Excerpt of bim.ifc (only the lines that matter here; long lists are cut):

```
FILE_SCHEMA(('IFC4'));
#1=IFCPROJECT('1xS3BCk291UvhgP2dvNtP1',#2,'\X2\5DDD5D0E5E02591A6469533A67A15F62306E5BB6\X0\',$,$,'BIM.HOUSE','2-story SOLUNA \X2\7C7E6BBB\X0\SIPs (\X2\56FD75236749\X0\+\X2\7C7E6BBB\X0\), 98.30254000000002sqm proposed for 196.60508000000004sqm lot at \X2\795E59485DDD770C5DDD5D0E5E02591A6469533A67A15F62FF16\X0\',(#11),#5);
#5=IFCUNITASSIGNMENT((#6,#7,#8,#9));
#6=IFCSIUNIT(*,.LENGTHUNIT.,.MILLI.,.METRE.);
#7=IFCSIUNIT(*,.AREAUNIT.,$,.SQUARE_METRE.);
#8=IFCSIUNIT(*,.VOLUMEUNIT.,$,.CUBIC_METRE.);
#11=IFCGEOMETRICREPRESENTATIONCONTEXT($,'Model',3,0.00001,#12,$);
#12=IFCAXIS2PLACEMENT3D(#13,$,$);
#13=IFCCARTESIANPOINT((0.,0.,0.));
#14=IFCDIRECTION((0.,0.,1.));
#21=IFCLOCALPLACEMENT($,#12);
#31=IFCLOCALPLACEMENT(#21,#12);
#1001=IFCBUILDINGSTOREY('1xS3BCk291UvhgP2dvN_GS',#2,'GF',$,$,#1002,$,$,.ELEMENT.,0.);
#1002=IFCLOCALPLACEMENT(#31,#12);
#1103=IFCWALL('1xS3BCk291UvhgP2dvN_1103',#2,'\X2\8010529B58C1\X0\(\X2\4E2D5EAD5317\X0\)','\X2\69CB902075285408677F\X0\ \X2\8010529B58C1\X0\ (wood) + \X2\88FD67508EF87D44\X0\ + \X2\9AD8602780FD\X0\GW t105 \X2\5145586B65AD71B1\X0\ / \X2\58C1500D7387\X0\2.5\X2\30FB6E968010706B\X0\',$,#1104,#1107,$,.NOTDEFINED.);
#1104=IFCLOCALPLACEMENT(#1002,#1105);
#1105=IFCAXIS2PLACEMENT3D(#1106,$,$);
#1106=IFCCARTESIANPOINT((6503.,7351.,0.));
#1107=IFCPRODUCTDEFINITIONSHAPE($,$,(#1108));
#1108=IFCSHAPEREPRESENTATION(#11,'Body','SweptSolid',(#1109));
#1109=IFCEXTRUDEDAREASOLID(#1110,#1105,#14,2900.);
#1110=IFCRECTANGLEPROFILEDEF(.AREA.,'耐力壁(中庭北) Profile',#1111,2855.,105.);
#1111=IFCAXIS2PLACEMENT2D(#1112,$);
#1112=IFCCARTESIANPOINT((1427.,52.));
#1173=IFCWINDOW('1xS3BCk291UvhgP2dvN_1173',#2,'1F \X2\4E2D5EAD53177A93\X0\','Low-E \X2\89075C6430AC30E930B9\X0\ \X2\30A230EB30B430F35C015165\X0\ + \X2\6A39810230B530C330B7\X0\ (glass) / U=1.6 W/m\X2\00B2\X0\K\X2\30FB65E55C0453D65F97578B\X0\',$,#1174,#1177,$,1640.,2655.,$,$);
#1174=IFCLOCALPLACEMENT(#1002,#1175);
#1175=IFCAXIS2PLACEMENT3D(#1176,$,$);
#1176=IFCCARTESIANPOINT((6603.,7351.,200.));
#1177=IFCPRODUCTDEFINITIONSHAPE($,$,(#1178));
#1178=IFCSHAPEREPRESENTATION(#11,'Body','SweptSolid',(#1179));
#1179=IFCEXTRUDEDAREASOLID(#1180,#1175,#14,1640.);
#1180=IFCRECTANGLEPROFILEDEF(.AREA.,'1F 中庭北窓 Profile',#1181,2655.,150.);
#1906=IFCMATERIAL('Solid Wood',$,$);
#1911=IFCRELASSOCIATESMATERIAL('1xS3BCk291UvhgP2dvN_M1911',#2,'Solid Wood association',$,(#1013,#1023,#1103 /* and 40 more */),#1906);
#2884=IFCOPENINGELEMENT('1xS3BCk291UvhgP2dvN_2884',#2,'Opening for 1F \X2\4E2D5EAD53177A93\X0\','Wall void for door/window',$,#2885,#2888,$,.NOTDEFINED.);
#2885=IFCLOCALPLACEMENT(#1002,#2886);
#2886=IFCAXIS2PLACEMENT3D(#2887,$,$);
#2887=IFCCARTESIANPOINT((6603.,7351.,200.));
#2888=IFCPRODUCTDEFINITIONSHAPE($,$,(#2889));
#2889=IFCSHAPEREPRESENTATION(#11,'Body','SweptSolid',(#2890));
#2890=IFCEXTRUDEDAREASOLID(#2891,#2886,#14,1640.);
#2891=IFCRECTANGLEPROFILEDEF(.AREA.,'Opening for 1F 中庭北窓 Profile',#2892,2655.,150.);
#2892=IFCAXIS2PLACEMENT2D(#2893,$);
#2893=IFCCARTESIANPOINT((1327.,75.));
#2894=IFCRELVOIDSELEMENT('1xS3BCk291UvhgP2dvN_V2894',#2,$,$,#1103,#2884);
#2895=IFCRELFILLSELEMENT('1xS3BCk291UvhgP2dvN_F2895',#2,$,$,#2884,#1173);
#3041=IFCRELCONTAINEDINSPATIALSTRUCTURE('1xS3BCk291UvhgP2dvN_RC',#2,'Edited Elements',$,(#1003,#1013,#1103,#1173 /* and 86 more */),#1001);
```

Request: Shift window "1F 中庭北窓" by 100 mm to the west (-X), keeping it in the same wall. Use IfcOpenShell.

```python
import ifcopenshell
import ifcopenshell.api.geometry
import ifcopenshell.util.placement
import ifcopenshell.util.unit

model = ifcopenshell.open("bim.ifc")
unit_scale = ifcopenshell.util.unit.calculate_unit_scale(model)

window = model.by_guid("1xS3BCk291UvhgP2dvN_1173")
opening = window.FillsVoids[0].RelatingOpeningElement
wall = opening.VoidsElements[0].RelatingBuildingElement

wall_matrix = ifcopenshell.util.placement.get_local_placement(wall.ObjectPlacement)
shift = wall_matrix[:3, 0] * -0.1 / unit_scale
before = ifcopenshell.util.placement.get_local_placement(window.ObjectPlacement)[:3, 3].copy()

# The window is not placed relative to its opening, so move both.
for product in (opening, window):
    matrix = ifcopenshell.util.placement.get_local_placement(product.ObjectPlacement)
    matrix[:3, 3] += shift
    ifcopenshell.api.geometry.edit_object_placement(model, product=product, matrix=matrix, is_si=False)

after = ifcopenshell.util.placement.get_local_placement(window.ObjectPlacement)[:3, 3]
print("window moved by", (after - before).round(3) + 0.0)

model.write("bim-out.ifc")
```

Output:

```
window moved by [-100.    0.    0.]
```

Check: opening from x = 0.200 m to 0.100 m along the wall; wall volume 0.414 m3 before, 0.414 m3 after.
